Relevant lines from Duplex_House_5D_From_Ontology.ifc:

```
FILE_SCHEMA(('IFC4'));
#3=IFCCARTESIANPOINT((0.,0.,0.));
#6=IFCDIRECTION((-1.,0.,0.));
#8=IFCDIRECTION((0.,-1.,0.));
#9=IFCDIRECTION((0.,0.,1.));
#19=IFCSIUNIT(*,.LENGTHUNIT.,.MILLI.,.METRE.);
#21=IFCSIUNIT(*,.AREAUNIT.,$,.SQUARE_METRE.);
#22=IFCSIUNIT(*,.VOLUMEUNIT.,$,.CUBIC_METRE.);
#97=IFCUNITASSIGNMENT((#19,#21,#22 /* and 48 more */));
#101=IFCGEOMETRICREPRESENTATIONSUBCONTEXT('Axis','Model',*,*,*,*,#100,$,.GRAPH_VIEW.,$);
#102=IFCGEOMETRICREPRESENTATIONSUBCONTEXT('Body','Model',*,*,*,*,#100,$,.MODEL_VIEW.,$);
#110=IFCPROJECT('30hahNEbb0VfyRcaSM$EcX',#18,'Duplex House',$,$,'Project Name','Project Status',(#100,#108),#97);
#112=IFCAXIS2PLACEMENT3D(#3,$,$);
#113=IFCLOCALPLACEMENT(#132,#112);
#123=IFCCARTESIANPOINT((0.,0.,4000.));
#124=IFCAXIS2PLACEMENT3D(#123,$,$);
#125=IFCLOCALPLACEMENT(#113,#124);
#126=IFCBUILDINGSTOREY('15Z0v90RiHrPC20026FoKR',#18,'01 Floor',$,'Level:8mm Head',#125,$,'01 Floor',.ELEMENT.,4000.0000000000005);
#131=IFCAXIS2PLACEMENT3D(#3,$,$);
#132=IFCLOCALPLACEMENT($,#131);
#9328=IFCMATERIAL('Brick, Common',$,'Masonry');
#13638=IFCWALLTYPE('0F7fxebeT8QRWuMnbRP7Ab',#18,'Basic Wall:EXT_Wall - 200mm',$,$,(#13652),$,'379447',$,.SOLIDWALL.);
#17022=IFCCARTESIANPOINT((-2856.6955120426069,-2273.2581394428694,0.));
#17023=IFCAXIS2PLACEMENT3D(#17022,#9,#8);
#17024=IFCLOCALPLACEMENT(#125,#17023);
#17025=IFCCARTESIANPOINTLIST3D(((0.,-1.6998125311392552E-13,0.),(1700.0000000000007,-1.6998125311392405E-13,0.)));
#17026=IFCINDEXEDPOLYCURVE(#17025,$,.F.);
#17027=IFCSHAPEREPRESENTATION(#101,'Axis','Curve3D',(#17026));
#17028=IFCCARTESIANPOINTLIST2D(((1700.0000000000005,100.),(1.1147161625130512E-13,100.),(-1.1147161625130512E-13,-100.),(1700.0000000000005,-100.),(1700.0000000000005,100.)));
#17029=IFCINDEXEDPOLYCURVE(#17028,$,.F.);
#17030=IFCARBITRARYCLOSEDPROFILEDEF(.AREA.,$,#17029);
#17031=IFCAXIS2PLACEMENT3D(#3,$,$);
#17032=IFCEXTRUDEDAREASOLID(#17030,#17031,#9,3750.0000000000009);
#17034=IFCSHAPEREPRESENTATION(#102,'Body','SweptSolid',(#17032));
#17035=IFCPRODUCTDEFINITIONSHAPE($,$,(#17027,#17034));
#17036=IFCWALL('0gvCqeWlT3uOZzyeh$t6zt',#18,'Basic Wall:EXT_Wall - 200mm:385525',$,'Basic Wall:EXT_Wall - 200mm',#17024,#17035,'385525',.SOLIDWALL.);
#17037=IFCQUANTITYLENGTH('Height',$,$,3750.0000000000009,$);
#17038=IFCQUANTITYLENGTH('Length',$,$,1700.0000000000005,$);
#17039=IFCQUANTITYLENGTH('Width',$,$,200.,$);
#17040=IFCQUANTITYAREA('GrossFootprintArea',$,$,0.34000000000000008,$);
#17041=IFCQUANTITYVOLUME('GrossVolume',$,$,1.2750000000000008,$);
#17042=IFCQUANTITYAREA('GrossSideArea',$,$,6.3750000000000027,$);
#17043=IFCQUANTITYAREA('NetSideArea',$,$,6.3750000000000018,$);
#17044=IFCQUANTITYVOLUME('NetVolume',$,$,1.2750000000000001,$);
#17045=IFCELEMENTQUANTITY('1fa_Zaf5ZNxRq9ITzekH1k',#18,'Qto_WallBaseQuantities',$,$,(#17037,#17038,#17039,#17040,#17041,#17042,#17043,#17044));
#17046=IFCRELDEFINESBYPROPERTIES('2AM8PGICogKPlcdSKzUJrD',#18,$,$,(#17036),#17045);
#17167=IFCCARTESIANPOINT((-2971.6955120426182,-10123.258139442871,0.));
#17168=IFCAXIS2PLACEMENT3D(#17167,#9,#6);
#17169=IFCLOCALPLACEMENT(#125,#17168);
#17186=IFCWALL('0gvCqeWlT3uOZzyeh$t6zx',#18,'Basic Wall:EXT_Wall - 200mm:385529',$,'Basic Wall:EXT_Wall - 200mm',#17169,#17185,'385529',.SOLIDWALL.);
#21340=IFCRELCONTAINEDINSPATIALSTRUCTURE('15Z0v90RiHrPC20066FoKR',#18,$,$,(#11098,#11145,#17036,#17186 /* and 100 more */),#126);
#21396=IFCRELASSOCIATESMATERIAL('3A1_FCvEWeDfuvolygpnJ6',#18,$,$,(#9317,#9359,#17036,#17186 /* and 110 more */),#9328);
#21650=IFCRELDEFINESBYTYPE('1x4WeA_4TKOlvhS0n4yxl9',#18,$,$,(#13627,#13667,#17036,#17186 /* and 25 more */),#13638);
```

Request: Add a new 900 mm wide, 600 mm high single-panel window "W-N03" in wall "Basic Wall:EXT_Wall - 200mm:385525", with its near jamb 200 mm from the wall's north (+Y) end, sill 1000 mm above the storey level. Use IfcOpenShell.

```python
import numpy as np
import ifcopenshell
import ifcopenshell.api.feature
import ifcopenshell.api.geometry
import ifcopenshell.api.pset
import ifcopenshell.api.root
import ifcopenshell.api.spatial
import ifcopenshell.geom
import ifcopenshell.util.element
import ifcopenshell.util.placement
import ifcopenshell.util.representation
import ifcopenshell.util.shape
import ifcopenshell.util.unit

model = ifcopenshell.open("Duplex_House_5D_From_Ontology.ifc")
unit_scale = ifcopenshell.util.unit.calculate_unit_scale(model)
area_scale = ifcopenshell.util.unit.calculate_unit_scale(model, "AREAUNIT")
volume_scale = ifcopenshell.util.unit.calculate_unit_scale(model, "VOLUMEUNIT")
settings = ifcopenshell.geom.settings()


def volume(element):
    """Net volume in cubic metres, openings subtracted."""
    shape = ifcopenshell.geom.create_shape(settings, element)
    return ifcopenshell.util.shape.get_volume(shape.geometry)


wall = model.by_guid("0gvCqeWlT3uOZzyeh$t6zt")
storey = ifcopenshell.util.element.get_container(wall, ifc_class="IfcBuildingStorey")
context = ifcopenshell.util.representation.get_context(model, "Model", "Body", "MODEL_VIEW")
before = volume(wall)

width, height, from_end, sill = 0.9, 0.6, 0.2, 1  # metres

# The wall runs along its own X axis, and the end named is its -X end.
wall_shape = ifcopenshell.geom.create_shape(settings, wall)
x, y, z = ifcopenshell.util.shape.get_vertices(wall_shape.geometry).T
start = x.min() + from_end
face, thickness = float(y.min()), float(y.max() - y.min())
wall_matrix = ifcopenshell.util.placement.get_local_placement(wall.ObjectPlacement)
level = ifcopenshell.util.placement.get_local_placement(storey.ObjectPlacement)[2, 3]


def in_wall(x, y):
    """Placement at x, y metres in the wall's axes, at sill height."""
    matrix = wall_matrix.copy()
    matrix[:, 3] = wall_matrix @ np.array([x / unit_scale, y / unit_scale, 0.0, 1.0])
    matrix[2, 3] = level + sill / unit_scale
    return matrix


# Opening: a box that overshoots both wall faces by 50 mm.
opening = ifcopenshell.api.root.create_entity(model, ifc_class="IfcOpeningElement", predefined_type="OPENING")
box = ifcopenshell.api.geometry.add_wall_representation(
    model, context=context, length=width, height=height, thickness=thickness + 0.1
)
ifcopenshell.api.geometry.assign_representation(model, product=opening, representation=box)
ifcopenshell.api.geometry.edit_object_placement(model, product=opening, matrix=in_wall(start, face - 0.05), is_si=False)
ifcopenshell.api.feature.add_feature(model, feature=opening, element=wall)

window = ifcopenshell.api.root.create_entity(model, ifc_class="IfcWindow", name="W-N03", predefined_type="WINDOW")
window.OverallWidth, window.OverallHeight = width / unit_scale, height / unit_scale
window.PartitioningType = "SINGLE_PANEL"
body = ifcopenshell.api.geometry.add_window_representation(
    model,
    context=context,
    overall_width=window.OverallWidth,
    overall_height=window.OverallHeight,
    partition_type="SINGLE_PANEL",
)
ifcopenshell.api.geometry.assign_representation(model, product=window, representation=body)
ifcopenshell.api.spatial.assign_container(model, products=[window], relating_structure=storey)
ifcopenshell.api.feature.add_filling(model, opening=opening, element=window)

# Centre the window in the wall's thickness.
ifcopenshell.api.geometry.edit_object_placement(model, product=window, matrix=in_wall(start, face), is_si=False)
window_shape = ifcopenshell.geom.create_shape(settings, window)
depth = ifcopenshell.util.shape.get_vertices(window_shape.geometry)[:, 1]
offset = face + thickness / 2 - (depth.min() + depth.max()) / 2
ifcopenshell.api.geometry.edit_object_placement(model, product=window, matrix=in_wall(start, offset), is_si=False)

after = volume(wall)

# Update the wall's stored quantities.
qto = model.by_id(ifcopenshell.util.element.get_pset(wall, "Qto_WallBaseQuantities", should_inherit=False)["id"])
ifcopenshell.api.pset.edit_qto(model, qto=qto, properties={
    "NetSideArea": after / thickness / area_scale,
    "NetVolume": after / volume_scale,
})

print(f"wall volume {before:.3f} -> {after:.3f} m3")

model.write("Duplex_House_5D_From_Ontology_updated.ifc")
```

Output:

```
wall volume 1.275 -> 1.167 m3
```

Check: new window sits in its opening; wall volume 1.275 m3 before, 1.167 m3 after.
